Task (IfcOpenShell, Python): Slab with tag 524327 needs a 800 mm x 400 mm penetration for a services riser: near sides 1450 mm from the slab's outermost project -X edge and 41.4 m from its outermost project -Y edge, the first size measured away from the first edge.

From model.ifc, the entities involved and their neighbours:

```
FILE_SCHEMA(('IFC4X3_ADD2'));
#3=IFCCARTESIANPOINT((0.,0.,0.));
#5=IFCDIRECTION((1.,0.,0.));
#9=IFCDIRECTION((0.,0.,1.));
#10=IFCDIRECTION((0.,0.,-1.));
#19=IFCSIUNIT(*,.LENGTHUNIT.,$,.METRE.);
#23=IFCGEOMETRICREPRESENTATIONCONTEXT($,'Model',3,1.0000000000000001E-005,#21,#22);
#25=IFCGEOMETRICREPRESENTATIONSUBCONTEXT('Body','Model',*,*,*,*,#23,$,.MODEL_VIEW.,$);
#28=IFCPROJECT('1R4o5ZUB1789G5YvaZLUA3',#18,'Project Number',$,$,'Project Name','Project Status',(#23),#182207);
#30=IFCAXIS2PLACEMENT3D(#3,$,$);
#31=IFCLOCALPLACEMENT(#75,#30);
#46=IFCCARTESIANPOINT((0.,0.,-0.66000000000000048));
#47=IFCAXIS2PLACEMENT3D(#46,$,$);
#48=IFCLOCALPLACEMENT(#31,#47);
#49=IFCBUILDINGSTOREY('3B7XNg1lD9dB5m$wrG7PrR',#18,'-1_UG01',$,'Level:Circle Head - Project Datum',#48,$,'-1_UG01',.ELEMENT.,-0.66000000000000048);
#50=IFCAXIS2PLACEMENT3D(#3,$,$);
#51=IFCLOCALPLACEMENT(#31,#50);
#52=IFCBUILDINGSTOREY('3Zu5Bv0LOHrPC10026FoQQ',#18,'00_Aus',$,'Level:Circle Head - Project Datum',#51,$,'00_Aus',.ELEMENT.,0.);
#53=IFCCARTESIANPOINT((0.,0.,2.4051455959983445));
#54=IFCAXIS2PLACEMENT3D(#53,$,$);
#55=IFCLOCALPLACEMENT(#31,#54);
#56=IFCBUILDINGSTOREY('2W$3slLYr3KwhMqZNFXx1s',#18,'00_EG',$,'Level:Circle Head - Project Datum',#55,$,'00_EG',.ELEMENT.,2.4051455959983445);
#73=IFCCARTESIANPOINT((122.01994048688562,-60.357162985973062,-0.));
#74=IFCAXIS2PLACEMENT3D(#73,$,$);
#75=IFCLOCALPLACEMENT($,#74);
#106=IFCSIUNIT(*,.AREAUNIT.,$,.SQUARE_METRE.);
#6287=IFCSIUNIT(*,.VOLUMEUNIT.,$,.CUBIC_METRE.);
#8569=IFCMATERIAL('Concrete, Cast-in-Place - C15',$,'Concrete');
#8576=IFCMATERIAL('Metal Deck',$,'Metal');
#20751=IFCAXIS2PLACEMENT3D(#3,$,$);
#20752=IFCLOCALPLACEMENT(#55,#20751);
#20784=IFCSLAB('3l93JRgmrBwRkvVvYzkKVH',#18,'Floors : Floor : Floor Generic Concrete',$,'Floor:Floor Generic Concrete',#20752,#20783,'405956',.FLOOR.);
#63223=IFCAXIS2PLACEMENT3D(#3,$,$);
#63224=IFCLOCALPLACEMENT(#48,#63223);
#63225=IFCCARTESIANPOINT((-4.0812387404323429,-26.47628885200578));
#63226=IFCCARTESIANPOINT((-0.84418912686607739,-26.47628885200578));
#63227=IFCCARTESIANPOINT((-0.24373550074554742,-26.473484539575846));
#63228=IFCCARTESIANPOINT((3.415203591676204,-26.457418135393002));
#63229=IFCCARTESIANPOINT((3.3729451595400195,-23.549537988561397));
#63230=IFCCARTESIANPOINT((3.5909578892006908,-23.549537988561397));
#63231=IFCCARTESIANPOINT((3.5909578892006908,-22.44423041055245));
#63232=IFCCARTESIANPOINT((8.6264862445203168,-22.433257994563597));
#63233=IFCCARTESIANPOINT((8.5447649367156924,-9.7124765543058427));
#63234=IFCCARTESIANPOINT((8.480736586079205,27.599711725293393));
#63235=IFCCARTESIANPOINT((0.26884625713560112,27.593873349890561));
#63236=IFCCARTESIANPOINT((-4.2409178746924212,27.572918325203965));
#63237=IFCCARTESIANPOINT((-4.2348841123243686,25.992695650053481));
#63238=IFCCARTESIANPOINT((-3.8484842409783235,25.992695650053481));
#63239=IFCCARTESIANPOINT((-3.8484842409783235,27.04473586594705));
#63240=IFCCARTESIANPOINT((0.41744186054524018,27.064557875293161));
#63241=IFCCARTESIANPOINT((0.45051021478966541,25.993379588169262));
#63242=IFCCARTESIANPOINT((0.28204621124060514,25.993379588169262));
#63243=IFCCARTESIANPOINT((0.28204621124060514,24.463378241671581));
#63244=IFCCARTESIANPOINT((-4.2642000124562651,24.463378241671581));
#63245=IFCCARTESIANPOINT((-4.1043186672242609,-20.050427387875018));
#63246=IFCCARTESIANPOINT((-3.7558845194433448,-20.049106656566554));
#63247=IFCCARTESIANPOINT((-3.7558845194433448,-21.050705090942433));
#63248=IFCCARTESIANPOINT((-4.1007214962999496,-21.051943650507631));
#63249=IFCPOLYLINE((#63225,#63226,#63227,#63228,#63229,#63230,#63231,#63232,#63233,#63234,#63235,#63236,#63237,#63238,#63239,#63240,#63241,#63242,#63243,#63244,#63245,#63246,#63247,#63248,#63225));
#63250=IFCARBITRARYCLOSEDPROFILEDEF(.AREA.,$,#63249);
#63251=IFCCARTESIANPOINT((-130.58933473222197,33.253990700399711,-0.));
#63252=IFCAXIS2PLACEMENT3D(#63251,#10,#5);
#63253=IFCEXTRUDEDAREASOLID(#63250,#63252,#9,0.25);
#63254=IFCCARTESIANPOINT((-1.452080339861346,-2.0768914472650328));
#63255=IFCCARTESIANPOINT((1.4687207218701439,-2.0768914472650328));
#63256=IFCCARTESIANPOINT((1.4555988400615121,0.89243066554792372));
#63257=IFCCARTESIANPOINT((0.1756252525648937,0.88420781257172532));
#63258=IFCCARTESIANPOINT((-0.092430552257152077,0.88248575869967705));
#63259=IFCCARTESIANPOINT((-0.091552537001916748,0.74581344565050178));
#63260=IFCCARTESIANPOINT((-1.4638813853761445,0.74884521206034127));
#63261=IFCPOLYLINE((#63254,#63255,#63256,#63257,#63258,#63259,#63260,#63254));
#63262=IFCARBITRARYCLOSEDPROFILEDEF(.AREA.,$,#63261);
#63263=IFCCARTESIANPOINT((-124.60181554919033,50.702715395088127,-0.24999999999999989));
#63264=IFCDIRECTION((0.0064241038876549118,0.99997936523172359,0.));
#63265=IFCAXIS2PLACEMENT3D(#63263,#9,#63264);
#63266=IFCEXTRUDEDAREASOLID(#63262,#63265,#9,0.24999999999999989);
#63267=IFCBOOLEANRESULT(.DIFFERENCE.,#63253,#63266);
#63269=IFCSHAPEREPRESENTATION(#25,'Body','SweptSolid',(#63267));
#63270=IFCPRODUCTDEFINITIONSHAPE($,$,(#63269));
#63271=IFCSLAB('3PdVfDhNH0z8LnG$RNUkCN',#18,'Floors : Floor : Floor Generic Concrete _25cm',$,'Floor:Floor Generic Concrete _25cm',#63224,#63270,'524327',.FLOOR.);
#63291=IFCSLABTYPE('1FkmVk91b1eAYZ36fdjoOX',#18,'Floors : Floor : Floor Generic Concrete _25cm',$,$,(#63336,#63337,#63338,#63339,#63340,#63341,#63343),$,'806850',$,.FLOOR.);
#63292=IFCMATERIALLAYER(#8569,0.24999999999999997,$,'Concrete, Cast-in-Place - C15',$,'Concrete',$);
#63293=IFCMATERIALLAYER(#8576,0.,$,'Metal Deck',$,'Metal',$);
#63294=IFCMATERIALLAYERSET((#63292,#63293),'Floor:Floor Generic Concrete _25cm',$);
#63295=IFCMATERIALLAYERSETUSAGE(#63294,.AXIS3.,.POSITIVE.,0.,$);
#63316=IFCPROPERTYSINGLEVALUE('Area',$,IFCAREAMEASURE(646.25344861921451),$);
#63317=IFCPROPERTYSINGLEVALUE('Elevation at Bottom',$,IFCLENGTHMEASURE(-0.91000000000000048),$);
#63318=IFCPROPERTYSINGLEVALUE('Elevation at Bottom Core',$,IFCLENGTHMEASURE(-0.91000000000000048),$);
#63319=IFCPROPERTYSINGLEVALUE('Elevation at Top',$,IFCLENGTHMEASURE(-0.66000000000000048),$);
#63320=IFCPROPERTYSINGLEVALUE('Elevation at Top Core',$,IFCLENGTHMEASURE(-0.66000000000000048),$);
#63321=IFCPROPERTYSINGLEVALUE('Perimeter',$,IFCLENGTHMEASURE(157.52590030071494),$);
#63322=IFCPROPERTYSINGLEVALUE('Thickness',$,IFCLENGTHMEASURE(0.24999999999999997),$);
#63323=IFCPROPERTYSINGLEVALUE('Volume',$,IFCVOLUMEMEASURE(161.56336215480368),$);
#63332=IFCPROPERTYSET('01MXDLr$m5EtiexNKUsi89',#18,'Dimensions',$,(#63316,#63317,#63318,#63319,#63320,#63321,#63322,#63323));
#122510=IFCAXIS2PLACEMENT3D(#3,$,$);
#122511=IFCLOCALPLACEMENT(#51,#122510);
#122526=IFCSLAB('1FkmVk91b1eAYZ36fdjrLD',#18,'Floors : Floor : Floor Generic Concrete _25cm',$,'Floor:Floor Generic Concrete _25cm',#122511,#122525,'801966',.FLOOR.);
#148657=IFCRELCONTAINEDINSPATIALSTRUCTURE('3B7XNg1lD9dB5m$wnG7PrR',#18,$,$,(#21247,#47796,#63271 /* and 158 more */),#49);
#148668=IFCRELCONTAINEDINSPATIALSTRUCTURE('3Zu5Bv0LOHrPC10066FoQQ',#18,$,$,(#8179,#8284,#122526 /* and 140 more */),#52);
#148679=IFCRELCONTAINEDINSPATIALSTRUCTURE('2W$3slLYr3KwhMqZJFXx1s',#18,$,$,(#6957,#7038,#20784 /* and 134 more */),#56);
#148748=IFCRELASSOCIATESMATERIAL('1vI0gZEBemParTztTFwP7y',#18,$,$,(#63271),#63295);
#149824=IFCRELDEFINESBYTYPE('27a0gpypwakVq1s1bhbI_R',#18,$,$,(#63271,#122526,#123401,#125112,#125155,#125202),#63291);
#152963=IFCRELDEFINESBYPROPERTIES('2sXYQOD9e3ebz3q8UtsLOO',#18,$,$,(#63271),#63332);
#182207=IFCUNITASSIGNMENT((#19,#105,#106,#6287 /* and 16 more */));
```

```python
import numpy as np
import ifcopenshell
import ifcopenshell.api.feature
import ifcopenshell.api.geometry
import ifcopenshell.api.pset
import ifcopenshell.api.root
import ifcopenshell.geom
import ifcopenshell.util.element
import ifcopenshell.util.placement
import ifcopenshell.util.representation
import ifcopenshell.util.shape
import ifcopenshell.util.unit

model = ifcopenshell.open("model.ifc")
unit_scale = ifcopenshell.util.unit.calculate_unit_scale(model)
area_scale = ifcopenshell.util.unit.calculate_unit_scale(model, "AREAUNIT")
volume_scale = ifcopenshell.util.unit.calculate_unit_scale(model, "VOLUMEUNIT")
settings = ifcopenshell.geom.settings()


def volume(element):
    """Net volume in cubic metres, openings subtracted."""
    shape = ifcopenshell.geom.create_shape(settings, element)
    return ifcopenshell.util.shape.get_volume(shape.geometry)


slab = model.by_guid("3PdVfDhNH0z8LnG$RNUkCN")
before = volume(slab)

# Extent in the slab's own axes, in metres. The edges named are its -X and -Y sides.
slab_shape = ifcopenshell.geom.create_shape(settings, slab)
vertices = ifcopenshell.util.shape.get_vertices(slab_shape.geometry)
x_min, y_min, bottom = vertices.min(axis=0)
top = vertices[:, 2].max()

opening = ifcopenshell.api.root.create_entity(model, ifc_class="IfcOpeningElement", name="Services riser opening", predefined_type="OPENING")
context = ifcopenshell.util.representation.get_context(model, "Model", "Body", "MODEL_VIEW")
width, depth = 0.8, 0.4
outline = [(0.0, 0.0), (width, 0.0), (width, depth), (0.0, depth), (0.0, 0.0)]
# Overshoot both faces by 50 mm so the cut is clean.
shape = ifcopenshell.api.geometry.add_slab_representation(
    model, context=context, depth=top - bottom + 0.1, polyline=outline
)
ifcopenshell.api.geometry.assign_representation(model, product=opening, representation=shape)

matrix = ifcopenshell.util.placement.get_local_placement(slab.ObjectPlacement)
matrix[:, 3] = matrix @ np.append(np.array([x_min + 1.45, y_min + 41.4, bottom - 0.05]) / unit_scale, 1.0)
ifcopenshell.api.geometry.edit_object_placement(model, product=opening, matrix=matrix, is_si=False)
ifcopenshell.api.feature.add_feature(model, feature=opening, element=slab)

after = volume(slab)

# Update the slab's stored quantities.
pset = model.by_id(ifcopenshell.util.element.get_pset(slab, "Dimensions", should_inherit=False)["id"])
ifcopenshell.api.pset.edit_pset(model, pset=pset, properties={
    "Area": model.create_entity("IfcAreaMeasure", after / (top - bottom) / area_scale),
    "Volume": model.create_entity("IfcVolumeMeasure", after / volume_scale),
})

print(f"slab volume {before:.3f} -> {after:.3f} m3")

model.write("model_rev.ifc")
```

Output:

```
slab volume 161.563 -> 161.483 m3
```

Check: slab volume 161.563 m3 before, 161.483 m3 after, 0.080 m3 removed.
